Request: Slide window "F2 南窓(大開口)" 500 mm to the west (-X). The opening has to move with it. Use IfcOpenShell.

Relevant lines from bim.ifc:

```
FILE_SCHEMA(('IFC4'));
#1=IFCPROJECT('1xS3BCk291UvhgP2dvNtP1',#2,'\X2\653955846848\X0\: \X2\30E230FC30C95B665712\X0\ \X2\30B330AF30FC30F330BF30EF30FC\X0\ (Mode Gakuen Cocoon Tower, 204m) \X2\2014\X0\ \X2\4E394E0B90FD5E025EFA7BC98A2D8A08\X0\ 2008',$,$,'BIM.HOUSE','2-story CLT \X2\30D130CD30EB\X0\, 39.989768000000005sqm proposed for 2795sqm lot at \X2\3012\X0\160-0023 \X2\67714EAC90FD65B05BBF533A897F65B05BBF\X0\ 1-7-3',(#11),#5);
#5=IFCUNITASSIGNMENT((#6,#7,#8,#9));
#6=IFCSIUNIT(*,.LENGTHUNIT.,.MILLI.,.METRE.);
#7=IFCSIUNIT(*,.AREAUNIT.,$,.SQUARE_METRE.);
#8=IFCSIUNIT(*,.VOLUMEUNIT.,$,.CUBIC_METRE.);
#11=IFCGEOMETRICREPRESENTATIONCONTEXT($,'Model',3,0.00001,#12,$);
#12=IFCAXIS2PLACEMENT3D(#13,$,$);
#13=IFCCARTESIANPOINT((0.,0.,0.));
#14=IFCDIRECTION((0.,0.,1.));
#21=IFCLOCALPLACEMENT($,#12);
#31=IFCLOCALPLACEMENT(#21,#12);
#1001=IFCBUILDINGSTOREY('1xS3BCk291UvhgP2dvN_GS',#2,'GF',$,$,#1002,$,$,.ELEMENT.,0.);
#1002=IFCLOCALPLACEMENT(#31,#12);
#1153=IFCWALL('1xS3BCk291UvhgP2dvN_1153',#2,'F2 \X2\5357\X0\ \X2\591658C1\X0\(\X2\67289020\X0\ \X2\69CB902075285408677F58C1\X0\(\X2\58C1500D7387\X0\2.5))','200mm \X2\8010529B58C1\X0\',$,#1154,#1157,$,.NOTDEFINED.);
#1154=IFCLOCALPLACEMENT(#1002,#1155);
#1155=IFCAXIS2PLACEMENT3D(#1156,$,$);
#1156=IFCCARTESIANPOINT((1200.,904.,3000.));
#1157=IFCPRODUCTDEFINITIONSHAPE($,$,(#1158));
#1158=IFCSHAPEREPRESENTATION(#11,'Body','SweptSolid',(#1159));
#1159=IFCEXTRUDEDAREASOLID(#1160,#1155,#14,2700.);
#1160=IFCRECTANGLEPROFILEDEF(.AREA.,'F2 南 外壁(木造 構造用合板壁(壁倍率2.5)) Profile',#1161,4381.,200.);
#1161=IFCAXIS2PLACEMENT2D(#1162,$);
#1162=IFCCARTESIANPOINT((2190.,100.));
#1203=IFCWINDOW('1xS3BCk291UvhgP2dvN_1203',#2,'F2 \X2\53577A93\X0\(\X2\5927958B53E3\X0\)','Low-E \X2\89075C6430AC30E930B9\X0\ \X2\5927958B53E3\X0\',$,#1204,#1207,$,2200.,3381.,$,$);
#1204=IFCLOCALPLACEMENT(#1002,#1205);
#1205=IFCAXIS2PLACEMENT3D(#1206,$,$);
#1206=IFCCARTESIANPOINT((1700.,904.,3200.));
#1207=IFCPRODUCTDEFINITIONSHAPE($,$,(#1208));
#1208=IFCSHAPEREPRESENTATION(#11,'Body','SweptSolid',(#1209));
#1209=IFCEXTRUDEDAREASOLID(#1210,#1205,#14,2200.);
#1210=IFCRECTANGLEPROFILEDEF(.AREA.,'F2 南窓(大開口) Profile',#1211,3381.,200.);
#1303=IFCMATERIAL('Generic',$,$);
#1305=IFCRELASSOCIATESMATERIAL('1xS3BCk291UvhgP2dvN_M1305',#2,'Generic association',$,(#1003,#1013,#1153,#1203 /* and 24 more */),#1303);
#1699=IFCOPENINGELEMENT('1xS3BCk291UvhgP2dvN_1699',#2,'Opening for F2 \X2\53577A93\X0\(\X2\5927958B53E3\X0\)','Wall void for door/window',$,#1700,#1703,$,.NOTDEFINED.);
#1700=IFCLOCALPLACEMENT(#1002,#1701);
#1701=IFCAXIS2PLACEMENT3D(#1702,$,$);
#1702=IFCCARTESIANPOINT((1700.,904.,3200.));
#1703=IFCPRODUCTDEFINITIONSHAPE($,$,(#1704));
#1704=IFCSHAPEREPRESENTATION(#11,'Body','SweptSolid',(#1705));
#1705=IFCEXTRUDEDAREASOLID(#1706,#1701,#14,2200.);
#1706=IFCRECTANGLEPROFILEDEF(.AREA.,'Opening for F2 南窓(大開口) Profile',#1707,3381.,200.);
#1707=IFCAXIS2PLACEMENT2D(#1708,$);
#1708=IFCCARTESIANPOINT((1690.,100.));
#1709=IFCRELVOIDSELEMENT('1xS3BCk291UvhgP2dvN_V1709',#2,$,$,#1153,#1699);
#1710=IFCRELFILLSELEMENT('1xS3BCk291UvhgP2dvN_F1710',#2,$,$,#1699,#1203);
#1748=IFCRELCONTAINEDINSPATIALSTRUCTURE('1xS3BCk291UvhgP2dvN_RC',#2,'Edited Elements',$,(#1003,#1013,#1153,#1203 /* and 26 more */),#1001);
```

```python
import ifcopenshell
import ifcopenshell.api.geometry
import ifcopenshell.util.placement
import ifcopenshell.util.unit

model = ifcopenshell.open("bim.ifc")
unit_scale = ifcopenshell.util.unit.calculate_unit_scale(model)

window = model.by_guid("1xS3BCk291UvhgP2dvN_1203")
opening = window.FillsVoids[0].RelatingOpeningElement
wall = opening.VoidsElements[0].RelatingBuildingElement

wall_matrix = ifcopenshell.util.placement.get_local_placement(wall.ObjectPlacement)
shift = wall_matrix[:3, 0] * -0.5 / unit_scale
before = ifcopenshell.util.placement.get_local_placement(window.ObjectPlacement)[:3, 3].copy()

# The window is not placed relative to its opening, so move both.
for product in (opening, window):
    matrix = ifcopenshell.util.placement.get_local_placement(product.ObjectPlacement)
    matrix[:3, 3] += shift
    ifcopenshell.api.geometry.edit_object_placement(model, product=product, matrix=matrix, is_si=False)

after = ifcopenshell.util.placement.get_local_placement(window.ObjectPlacement)[:3, 3]
print("window moved by", (after - before).round(3) + 0.0)

model.write("bim_rev.ifc")
```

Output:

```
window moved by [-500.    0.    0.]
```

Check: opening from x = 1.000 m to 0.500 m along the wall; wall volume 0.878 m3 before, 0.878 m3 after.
